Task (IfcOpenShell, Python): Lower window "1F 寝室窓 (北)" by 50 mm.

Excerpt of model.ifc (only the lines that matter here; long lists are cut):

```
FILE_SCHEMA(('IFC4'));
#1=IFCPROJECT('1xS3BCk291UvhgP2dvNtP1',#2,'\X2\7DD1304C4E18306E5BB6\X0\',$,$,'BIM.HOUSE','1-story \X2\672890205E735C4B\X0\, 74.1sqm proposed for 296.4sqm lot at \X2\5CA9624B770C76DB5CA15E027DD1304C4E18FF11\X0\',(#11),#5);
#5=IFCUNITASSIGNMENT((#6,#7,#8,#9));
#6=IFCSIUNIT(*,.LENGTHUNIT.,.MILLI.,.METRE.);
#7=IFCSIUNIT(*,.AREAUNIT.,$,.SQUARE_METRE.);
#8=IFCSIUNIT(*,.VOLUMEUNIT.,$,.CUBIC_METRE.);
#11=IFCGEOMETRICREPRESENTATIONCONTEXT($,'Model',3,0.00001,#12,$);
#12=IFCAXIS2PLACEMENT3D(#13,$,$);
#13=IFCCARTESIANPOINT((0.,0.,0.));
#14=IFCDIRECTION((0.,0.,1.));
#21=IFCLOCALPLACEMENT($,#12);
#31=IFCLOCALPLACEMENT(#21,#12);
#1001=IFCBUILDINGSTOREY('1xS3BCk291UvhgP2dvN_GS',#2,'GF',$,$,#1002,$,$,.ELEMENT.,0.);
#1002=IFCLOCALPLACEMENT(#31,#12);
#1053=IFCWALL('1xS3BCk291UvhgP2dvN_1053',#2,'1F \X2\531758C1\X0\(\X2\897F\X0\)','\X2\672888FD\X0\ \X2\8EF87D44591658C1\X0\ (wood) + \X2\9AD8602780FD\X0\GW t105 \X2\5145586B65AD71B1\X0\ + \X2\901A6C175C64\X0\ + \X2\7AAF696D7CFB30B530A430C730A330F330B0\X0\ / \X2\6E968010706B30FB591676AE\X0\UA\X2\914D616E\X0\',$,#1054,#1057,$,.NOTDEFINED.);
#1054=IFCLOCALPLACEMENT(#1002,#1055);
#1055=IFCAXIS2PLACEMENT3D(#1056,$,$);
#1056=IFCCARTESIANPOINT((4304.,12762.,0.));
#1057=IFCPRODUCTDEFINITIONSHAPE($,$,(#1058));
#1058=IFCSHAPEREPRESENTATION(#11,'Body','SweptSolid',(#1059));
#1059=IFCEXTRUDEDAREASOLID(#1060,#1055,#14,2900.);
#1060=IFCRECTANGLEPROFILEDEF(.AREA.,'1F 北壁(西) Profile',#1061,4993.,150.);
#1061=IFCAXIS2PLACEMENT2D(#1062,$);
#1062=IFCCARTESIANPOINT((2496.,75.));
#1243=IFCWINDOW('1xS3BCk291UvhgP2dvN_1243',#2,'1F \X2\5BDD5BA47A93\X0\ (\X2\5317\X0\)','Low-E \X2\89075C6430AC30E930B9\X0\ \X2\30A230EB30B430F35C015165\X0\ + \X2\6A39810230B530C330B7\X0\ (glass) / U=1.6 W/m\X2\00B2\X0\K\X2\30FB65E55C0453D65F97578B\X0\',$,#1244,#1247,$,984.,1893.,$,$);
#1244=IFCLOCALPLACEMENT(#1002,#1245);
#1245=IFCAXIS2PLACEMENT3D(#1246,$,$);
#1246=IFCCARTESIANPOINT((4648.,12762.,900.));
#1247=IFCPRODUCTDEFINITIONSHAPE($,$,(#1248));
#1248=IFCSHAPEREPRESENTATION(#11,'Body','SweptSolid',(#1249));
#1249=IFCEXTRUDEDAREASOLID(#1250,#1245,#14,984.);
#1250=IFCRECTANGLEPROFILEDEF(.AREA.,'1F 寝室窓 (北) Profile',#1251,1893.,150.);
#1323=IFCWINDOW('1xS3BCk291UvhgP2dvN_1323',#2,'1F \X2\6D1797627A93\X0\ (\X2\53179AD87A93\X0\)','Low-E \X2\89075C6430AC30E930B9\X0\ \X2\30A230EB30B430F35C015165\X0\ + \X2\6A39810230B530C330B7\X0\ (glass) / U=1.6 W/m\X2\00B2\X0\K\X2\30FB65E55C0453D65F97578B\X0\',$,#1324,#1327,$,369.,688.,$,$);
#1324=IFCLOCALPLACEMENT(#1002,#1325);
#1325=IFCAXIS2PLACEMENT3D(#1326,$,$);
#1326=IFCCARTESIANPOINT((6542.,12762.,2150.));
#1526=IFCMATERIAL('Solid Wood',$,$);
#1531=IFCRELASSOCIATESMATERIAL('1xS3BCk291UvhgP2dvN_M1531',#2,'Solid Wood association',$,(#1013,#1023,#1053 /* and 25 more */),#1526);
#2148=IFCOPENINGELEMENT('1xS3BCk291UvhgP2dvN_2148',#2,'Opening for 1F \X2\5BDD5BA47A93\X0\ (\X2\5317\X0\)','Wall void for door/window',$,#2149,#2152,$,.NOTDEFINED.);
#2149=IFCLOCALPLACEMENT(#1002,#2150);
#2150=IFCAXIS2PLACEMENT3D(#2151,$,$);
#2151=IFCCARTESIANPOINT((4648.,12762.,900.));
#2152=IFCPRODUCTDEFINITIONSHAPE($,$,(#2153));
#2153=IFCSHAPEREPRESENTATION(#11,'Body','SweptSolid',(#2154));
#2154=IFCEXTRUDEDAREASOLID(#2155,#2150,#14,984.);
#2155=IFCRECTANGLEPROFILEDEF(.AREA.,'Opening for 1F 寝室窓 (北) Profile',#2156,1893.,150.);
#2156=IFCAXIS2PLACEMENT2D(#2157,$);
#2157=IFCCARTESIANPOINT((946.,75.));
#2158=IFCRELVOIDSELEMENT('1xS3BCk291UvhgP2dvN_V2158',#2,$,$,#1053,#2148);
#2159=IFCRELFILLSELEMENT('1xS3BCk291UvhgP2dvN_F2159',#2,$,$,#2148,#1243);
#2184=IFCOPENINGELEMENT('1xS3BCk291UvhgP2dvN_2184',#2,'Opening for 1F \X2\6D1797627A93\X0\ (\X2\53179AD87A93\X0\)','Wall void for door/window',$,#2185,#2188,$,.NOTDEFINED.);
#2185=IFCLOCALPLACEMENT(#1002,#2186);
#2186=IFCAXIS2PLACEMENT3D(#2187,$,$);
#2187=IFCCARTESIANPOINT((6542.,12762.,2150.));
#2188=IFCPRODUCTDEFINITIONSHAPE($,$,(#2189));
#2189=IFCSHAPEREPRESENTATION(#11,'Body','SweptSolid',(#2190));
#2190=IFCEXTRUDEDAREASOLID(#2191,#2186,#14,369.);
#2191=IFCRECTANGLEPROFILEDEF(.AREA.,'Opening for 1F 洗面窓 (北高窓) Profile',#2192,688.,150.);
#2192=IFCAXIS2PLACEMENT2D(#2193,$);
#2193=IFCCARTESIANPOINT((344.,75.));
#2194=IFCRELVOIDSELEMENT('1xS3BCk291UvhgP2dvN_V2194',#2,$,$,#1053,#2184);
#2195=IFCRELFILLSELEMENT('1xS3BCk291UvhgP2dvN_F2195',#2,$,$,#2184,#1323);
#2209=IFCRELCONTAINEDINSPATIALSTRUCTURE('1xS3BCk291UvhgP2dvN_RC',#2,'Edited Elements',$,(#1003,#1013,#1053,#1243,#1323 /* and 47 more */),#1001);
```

```python
import numpy as np
import ifcopenshell
import ifcopenshell.api.geometry
import ifcopenshell.util.placement
import ifcopenshell.util.unit

model = ifcopenshell.open("model.ifc")
unit_scale = ifcopenshell.util.unit.calculate_unit_scale(model)

window = model.by_id(1243)
opening = window.FillsVoids[0].RelatingOpeningElement
dz = -0.05 / unit_scale

shift = np.array([0.0, 0.0, dz])
# The window is not placed relative to its opening, so move both.
for product in (opening, window):
    matrix = ifcopenshell.util.placement.get_local_placement(product.ObjectPlacement)
    matrix[:3, 3] += shift
    ifcopenshell.api.geometry.edit_object_placement(model, product=product, matrix=matrix, is_si=False)

print(f"moved by {dz * unit_scale:+.3f} m")

model.write("model-out.ifc")
```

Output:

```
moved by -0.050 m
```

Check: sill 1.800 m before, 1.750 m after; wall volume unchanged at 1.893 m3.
